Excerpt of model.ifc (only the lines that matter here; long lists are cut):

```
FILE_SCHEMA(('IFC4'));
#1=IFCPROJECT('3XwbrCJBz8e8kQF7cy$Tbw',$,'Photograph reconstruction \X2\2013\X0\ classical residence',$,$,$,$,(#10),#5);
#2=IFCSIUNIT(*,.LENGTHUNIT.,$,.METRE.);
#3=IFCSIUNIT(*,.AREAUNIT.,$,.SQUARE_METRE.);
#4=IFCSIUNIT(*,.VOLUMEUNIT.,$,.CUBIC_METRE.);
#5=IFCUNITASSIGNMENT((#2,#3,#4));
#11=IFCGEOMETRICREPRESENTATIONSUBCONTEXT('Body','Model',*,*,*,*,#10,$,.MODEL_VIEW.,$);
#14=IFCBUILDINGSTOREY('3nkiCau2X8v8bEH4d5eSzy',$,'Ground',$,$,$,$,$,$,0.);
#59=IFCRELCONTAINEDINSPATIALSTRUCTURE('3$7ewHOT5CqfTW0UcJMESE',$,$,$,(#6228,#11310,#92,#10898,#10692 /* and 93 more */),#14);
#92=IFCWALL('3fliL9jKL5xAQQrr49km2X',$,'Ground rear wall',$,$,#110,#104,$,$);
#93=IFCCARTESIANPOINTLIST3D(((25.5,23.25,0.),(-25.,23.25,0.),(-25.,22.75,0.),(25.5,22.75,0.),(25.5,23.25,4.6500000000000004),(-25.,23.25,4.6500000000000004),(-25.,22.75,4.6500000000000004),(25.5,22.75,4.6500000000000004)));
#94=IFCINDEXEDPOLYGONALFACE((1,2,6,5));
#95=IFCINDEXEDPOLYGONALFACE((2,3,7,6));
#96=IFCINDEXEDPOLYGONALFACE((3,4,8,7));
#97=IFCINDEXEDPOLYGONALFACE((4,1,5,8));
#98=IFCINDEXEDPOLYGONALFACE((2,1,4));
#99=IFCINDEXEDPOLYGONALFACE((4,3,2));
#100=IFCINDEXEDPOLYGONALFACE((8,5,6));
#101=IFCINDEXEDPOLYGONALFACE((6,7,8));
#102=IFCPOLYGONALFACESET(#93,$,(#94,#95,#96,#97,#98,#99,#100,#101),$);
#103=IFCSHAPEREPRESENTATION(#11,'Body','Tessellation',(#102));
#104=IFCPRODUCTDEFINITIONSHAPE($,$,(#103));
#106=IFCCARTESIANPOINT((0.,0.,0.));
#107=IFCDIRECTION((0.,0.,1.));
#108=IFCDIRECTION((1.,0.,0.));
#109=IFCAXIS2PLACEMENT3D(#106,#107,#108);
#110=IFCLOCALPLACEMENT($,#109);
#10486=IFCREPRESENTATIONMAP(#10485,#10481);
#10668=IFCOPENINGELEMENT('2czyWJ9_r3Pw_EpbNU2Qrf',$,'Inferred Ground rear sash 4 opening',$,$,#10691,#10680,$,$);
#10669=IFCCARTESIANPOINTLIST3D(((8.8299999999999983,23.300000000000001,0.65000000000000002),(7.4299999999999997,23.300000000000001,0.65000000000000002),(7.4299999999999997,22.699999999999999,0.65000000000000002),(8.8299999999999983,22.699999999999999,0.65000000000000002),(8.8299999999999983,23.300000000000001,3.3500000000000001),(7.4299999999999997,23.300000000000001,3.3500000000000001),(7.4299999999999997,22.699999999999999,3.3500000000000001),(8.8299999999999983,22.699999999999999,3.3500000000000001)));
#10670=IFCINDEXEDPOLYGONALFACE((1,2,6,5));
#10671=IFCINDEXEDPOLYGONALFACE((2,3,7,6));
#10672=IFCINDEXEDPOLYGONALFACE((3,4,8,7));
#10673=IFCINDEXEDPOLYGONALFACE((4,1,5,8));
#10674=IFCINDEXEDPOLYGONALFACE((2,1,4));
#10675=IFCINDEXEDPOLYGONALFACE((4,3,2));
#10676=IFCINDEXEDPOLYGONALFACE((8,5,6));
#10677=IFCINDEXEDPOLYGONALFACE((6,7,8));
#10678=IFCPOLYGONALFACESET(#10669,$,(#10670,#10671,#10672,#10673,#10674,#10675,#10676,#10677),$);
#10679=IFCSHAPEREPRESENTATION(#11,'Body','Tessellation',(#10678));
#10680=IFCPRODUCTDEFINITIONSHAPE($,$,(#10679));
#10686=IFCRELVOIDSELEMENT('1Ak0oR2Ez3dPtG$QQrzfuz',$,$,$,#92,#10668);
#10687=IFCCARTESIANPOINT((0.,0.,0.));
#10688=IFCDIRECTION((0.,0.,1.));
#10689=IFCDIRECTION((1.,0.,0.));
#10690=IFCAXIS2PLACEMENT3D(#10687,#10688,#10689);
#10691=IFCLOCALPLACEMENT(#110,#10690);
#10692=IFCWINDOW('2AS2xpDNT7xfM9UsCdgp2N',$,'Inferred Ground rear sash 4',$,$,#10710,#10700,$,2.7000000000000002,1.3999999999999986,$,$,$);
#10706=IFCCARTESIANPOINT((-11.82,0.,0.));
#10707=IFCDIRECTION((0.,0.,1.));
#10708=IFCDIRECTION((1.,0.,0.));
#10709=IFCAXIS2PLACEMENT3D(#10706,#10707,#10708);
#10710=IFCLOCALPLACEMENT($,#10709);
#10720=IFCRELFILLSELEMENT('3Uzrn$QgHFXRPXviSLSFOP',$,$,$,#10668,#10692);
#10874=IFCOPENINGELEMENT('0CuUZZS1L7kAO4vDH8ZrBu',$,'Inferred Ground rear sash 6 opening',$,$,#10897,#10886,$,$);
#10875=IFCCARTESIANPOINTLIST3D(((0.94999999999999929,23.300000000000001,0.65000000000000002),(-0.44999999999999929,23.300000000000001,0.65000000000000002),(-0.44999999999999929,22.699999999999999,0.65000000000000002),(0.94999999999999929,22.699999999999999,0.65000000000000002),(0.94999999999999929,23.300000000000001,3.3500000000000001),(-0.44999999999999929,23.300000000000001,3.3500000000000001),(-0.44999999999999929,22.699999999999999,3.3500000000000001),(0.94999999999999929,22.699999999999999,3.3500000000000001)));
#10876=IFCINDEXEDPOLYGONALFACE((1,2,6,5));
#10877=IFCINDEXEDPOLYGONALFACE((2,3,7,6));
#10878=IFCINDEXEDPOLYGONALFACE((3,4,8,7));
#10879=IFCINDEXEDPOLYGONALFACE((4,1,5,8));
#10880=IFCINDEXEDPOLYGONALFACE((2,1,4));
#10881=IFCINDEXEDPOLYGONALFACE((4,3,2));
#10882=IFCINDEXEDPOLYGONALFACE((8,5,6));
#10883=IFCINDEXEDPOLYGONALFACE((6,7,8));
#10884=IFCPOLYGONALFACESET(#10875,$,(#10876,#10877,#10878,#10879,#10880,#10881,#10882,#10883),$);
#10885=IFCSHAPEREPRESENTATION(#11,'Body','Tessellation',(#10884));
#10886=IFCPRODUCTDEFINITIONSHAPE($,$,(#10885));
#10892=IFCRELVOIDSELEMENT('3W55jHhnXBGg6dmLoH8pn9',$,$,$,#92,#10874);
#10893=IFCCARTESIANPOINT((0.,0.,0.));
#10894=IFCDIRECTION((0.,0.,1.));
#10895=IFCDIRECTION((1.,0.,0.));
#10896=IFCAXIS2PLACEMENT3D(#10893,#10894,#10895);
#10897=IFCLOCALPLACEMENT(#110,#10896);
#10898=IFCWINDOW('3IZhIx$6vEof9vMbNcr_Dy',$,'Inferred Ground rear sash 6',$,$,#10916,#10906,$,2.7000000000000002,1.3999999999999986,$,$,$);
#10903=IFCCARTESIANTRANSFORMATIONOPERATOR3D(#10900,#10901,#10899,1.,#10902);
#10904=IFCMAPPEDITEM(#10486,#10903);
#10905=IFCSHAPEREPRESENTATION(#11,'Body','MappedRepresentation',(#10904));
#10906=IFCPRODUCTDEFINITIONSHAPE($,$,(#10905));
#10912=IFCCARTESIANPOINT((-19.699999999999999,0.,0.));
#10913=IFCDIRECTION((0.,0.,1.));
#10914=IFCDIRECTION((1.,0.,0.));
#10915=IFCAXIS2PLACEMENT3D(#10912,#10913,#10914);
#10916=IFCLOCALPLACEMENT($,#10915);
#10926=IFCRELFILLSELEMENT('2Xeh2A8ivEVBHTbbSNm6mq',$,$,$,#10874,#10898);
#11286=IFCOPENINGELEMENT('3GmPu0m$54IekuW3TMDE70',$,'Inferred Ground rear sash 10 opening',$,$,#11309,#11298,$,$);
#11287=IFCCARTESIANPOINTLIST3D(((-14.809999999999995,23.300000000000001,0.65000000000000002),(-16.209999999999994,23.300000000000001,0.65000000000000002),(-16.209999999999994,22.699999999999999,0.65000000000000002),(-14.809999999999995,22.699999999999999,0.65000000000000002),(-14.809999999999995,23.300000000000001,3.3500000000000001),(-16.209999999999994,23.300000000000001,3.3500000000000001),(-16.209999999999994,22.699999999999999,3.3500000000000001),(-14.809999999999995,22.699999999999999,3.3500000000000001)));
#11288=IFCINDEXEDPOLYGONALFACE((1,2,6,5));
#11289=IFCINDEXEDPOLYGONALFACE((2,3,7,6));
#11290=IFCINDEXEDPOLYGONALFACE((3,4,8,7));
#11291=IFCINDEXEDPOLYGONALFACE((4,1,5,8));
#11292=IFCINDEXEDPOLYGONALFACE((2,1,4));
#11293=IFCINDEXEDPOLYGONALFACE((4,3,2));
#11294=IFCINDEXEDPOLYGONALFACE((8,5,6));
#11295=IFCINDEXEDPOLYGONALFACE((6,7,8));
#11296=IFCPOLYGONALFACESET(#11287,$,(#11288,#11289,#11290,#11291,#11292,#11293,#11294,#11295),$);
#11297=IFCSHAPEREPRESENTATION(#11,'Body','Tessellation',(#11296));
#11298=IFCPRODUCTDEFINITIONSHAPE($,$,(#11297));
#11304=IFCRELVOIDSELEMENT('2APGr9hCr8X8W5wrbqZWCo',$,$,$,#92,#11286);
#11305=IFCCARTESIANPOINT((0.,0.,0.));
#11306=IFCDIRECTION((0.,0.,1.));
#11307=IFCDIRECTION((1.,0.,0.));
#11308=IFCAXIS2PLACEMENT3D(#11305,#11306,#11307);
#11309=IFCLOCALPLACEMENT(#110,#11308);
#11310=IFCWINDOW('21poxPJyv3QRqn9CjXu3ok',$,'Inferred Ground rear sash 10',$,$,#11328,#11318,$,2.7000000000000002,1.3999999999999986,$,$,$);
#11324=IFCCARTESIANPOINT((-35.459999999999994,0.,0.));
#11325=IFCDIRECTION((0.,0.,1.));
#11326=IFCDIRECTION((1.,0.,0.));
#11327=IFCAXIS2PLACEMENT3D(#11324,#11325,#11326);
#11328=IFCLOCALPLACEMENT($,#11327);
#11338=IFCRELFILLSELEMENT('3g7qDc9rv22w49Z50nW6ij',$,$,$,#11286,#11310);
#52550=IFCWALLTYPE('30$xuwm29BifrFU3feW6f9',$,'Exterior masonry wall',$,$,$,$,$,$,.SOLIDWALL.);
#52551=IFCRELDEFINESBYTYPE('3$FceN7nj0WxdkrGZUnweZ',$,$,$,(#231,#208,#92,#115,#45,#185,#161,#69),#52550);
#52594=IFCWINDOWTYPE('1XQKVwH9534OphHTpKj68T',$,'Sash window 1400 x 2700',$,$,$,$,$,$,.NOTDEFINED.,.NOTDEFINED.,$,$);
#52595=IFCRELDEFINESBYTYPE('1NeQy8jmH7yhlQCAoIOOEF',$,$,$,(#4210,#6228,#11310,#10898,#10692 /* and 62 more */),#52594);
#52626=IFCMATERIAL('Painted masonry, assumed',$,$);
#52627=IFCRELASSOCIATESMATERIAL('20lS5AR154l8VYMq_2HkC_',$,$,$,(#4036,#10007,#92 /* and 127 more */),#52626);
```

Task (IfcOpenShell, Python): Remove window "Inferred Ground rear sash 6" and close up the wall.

```python
import ifcopenshell
import ifcopenshell.api.feature
import ifcopenshell.api.root
import ifcopenshell.geom
import ifcopenshell.util.shape

model = ifcopenshell.open("model.ifc")
settings = ifcopenshell.geom.settings()


def volume(element):
    """Net volume in cubic metres, openings subtracted."""
    shape = ifcopenshell.geom.create_shape(settings, element)
    return ifcopenshell.util.shape.get_volume(shape.geometry)


window = model.by_guid("3IZhIx$6vEof9vMbNcr_Dy")
opening = window.FillsVoids[0].RelatingOpeningElement
wall = opening.VoidsElements[0].RelatingBuildingElement
before = volume(wall)

ifcopenshell.api.root.remove_product(model, product=window)
ifcopenshell.api.feature.remove_feature(model, feature=opening)

after = volume(wall)

print(f"wall volume {before:.3f} -> {after:.3f} m3")

model.write("model_rev.ifc")
```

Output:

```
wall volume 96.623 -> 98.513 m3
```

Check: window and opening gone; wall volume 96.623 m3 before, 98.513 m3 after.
